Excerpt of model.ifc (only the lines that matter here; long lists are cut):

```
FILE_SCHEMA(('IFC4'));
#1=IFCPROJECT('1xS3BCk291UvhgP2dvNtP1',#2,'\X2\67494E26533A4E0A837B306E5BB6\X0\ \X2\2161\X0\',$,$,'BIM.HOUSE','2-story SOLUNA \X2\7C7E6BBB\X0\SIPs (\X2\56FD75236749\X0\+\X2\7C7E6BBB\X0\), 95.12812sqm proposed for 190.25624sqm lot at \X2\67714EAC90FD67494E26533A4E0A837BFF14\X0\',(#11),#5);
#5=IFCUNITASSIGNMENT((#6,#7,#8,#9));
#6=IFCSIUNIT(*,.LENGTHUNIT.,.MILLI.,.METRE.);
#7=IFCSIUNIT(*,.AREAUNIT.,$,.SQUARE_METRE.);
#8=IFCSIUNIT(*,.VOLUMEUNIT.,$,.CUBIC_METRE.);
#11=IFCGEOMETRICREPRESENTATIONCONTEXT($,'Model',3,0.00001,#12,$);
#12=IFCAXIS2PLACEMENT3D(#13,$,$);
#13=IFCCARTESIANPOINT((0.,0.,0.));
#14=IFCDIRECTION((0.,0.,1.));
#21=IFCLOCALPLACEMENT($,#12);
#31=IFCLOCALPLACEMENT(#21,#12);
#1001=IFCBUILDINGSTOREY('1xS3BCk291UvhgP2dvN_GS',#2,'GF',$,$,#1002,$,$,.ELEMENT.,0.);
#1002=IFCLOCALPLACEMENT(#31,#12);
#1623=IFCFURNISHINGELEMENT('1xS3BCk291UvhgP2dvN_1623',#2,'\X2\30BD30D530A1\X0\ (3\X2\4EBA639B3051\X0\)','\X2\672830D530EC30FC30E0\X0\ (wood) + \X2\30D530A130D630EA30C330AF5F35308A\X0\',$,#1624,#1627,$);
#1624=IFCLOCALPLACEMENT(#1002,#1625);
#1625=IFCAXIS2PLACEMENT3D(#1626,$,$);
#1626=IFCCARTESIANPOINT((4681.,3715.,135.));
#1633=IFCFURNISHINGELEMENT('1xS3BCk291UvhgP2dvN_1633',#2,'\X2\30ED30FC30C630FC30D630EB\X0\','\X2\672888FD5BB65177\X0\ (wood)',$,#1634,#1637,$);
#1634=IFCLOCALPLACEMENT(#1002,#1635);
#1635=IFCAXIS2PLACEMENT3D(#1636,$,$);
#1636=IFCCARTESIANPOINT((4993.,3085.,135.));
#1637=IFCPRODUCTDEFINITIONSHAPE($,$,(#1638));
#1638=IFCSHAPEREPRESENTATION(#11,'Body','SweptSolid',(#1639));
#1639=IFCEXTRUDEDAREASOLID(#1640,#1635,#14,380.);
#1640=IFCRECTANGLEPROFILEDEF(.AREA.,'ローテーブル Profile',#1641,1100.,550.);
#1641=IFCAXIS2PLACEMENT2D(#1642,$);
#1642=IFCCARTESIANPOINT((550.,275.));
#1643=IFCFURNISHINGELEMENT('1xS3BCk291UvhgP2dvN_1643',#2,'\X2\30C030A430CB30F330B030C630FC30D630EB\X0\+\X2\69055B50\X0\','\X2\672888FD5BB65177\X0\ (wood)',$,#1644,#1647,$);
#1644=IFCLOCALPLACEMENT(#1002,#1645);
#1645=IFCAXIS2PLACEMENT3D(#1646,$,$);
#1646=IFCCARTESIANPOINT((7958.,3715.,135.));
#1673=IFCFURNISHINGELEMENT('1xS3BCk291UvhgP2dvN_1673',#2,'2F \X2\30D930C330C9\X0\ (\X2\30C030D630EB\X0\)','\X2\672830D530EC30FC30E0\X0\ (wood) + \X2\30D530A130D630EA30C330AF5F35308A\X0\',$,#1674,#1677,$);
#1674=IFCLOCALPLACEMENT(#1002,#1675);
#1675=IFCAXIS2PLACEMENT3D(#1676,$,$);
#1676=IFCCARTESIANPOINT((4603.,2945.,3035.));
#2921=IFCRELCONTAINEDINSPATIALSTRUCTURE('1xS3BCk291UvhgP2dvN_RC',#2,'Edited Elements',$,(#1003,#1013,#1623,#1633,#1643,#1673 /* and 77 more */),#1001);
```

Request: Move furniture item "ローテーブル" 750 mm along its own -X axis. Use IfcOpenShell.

```python
import ifcopenshell
import ifcopenshell.api.geometry
import ifcopenshell.util.placement
import ifcopenshell.util.unit

model = ifcopenshell.open("model.ifc")
unit_scale = ifcopenshell.util.unit.calculate_unit_scale(model)

item = model.by_guid("1xS3BCk291UvhgP2dvN_1633")
matrix = ifcopenshell.util.placement.get_local_placement(item.ObjectPlacement)
matrix[:3, 3] -= matrix[:3, 0] * 0.75 / unit_scale
ifcopenshell.api.geometry.edit_object_placement(model, product=item, matrix=matrix, is_si=False)

print(ifcopenshell.util.placement.get_local_placement(item.ObjectPlacement).round(3) + 0.0)

model.write("model-out.ifc")
```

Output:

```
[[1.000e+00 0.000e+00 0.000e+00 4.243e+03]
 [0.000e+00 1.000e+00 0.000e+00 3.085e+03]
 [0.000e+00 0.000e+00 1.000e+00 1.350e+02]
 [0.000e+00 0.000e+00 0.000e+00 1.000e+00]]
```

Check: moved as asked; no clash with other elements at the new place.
